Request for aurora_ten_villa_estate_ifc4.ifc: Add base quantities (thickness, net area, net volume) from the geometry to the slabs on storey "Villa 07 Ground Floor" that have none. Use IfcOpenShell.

First a look at what the model holds.

```python
import ifcopenshell
import ifcopenshell.util.element
import ifcopenshell.util.unit

model = ifcopenshell.open("aurora_ten_villa_estate_ifc4.ifc")
print(model.schema)
for unit_type in ("LENGTHUNIT", "AREAUNIT", "VOLUMEUNIT"):
    print(unit_type, ifcopenshell.util.unit.calculate_unit_scale(model, unit_type))
storey = next(s for s in model.by_type("IfcBuildingStorey") if s.Name == "Villa 07 Ground Floor")
slabs = [e for e in ifcopenshell.util.element.get_decomposition(storey) if e.is_a("IfcSlab")]
for e in sorted(slabs, key=lambda e: e.id()):
    print(e.id(), e.is_a(), e.Name, list(ifcopenshell.util.element.get_psets(e, qtos_only=True)), sep=" | ")
```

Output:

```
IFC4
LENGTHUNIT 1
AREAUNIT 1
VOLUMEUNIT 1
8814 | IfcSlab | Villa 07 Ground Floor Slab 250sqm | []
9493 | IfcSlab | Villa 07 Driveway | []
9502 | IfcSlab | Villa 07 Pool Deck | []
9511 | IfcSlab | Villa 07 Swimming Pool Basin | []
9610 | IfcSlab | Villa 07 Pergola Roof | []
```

```python
import ifcopenshell
import ifcopenshell.api.pset
import ifcopenshell.geom
import ifcopenshell.util.element
import ifcopenshell.util.shape
import ifcopenshell.util.unit

model = ifcopenshell.open("aurora_ten_villa_estate_ifc4.ifc")
unit_scale = ifcopenshell.util.unit.calculate_unit_scale(model)
area_scale = ifcopenshell.util.unit.calculate_unit_scale(model, "AREAUNIT")
volume_scale = ifcopenshell.util.unit.calculate_unit_scale(model, "VOLUMEUNIT")
settings = ifcopenshell.geom.settings()

storey = next(s for s in model.by_type("IfcBuildingStorey") if s.Name == "Villa 07 Ground Floor")
slabs = [e for e in ifcopenshell.util.element.get_decomposition(storey) if e.is_a("IfcSlab")]

for e in sorted(slabs, key=lambda e: e.id()):
    if ifcopenshell.util.element.get_psets(e, qtos_only=True, should_inherit=False):
        continue
    # Geometry comes back in metres, in the element's own axes.
    shape = ifcopenshell.geom.create_shape(settings, e)
    values = {
        "Width": ifcopenshell.util.shape.get_z(shape.geometry) / unit_scale,
        "NetArea": ifcopenshell.util.shape.get_footprint_area(shape.geometry) / area_scale,
        "NetVolume": ifcopenshell.util.shape.get_volume(shape.geometry) / volume_scale,
    }
    qto = ifcopenshell.api.pset.add_qto(model, product=e, name="Qto_SlabBaseQuantities")
    ifcopenshell.api.pset.edit_qto(model, qto=qto, properties=values)
    print(e.id(), {k: round(v, 3) for k, v in values.items()})

model.write("aurora_ten_villa_estate_ifc4_rev.ifc")
```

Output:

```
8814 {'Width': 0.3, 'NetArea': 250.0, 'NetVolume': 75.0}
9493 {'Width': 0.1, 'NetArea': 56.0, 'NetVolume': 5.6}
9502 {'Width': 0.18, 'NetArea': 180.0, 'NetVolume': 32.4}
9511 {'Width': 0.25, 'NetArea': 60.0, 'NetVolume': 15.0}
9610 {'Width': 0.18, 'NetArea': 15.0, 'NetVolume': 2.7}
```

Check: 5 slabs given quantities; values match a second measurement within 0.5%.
